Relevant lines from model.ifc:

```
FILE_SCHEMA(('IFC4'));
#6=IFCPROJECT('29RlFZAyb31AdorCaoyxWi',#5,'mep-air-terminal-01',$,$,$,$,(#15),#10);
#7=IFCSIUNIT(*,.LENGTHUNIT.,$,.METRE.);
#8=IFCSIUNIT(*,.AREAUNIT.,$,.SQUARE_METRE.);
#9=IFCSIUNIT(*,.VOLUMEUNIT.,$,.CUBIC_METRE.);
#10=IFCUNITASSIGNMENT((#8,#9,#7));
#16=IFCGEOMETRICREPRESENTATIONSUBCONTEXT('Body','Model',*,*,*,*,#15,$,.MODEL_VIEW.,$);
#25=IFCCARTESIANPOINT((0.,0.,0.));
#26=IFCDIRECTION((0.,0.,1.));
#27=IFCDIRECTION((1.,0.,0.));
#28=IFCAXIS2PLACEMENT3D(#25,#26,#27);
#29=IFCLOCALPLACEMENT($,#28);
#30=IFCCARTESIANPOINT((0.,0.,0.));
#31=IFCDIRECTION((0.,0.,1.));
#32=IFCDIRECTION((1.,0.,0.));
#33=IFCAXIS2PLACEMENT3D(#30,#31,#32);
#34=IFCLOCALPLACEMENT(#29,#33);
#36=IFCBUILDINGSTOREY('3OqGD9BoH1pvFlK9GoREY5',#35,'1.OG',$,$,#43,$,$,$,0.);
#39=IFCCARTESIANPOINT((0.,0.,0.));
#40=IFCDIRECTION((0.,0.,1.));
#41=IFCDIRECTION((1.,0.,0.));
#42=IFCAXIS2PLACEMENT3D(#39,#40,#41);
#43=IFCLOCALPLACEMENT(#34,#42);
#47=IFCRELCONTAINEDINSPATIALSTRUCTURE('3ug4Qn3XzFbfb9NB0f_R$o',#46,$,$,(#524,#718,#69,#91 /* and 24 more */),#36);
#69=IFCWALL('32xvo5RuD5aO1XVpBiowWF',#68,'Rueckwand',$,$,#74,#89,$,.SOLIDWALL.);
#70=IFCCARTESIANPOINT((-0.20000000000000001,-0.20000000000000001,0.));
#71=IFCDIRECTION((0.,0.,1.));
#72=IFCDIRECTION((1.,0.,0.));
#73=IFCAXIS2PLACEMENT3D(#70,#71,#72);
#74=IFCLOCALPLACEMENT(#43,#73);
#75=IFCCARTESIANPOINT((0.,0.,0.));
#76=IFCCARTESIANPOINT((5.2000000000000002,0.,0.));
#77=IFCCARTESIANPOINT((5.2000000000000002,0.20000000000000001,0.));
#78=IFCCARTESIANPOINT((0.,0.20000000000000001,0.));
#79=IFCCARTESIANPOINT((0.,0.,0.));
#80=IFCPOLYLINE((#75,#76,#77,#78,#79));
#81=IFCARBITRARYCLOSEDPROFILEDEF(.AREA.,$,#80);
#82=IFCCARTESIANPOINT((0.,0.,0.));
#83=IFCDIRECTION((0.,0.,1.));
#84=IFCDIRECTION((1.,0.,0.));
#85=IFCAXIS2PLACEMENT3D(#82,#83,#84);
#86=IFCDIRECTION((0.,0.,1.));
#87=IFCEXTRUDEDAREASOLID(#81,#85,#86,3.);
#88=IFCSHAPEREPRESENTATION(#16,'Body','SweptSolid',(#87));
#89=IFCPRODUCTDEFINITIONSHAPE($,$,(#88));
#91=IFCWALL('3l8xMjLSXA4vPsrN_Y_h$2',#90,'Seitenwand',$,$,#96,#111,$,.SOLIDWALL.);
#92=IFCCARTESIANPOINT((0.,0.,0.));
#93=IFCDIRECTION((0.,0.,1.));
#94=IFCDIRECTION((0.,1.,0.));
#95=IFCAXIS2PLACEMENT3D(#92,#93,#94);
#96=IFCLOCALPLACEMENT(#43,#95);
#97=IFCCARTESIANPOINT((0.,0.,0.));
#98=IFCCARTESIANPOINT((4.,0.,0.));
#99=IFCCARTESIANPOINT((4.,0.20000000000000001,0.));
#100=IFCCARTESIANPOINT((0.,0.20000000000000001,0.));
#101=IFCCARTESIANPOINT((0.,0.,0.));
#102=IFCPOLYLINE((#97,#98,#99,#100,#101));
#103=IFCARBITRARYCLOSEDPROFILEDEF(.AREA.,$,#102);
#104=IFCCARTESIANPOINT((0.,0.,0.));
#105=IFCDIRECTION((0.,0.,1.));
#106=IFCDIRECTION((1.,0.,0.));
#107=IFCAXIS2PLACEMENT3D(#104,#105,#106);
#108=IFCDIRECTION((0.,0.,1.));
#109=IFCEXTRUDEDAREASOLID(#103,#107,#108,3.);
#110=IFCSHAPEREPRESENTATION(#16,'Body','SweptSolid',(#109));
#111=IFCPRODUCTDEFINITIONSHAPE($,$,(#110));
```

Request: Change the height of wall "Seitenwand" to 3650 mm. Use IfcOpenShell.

```python
import ifcopenshell
import ifcopenshell.geom
import ifcopenshell.util.representation
import ifcopenshell.util.shape
import ifcopenshell.util.unit

model = ifcopenshell.open("model.ifc")
unit_scale = ifcopenshell.util.unit.calculate_unit_scale(model)
settings = ifcopenshell.geom.settings()


def volume(element):
    """Net volume in cubic metres, openings subtracted."""
    shape = ifcopenshell.geom.create_shape(settings, element)
    return ifcopenshell.util.shape.get_volume(shape.geometry)


wall = model.by_id(91)
before = volume(wall)

body = ifcopenshell.util.representation.get_representation(wall, "Model", "Body")
solid = body.Items[0]
old_height = solid.Depth
solid.Depth = 3.65 / unit_scale
after = volume(wall)

print(f"height {old_height:g} -> {solid.Depth:g}, volume {before:.3f} -> {after:.3f} m3")

model.write("model_v2.ifc")
```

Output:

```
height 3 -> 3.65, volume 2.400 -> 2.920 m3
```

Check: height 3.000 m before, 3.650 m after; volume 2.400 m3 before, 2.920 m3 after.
